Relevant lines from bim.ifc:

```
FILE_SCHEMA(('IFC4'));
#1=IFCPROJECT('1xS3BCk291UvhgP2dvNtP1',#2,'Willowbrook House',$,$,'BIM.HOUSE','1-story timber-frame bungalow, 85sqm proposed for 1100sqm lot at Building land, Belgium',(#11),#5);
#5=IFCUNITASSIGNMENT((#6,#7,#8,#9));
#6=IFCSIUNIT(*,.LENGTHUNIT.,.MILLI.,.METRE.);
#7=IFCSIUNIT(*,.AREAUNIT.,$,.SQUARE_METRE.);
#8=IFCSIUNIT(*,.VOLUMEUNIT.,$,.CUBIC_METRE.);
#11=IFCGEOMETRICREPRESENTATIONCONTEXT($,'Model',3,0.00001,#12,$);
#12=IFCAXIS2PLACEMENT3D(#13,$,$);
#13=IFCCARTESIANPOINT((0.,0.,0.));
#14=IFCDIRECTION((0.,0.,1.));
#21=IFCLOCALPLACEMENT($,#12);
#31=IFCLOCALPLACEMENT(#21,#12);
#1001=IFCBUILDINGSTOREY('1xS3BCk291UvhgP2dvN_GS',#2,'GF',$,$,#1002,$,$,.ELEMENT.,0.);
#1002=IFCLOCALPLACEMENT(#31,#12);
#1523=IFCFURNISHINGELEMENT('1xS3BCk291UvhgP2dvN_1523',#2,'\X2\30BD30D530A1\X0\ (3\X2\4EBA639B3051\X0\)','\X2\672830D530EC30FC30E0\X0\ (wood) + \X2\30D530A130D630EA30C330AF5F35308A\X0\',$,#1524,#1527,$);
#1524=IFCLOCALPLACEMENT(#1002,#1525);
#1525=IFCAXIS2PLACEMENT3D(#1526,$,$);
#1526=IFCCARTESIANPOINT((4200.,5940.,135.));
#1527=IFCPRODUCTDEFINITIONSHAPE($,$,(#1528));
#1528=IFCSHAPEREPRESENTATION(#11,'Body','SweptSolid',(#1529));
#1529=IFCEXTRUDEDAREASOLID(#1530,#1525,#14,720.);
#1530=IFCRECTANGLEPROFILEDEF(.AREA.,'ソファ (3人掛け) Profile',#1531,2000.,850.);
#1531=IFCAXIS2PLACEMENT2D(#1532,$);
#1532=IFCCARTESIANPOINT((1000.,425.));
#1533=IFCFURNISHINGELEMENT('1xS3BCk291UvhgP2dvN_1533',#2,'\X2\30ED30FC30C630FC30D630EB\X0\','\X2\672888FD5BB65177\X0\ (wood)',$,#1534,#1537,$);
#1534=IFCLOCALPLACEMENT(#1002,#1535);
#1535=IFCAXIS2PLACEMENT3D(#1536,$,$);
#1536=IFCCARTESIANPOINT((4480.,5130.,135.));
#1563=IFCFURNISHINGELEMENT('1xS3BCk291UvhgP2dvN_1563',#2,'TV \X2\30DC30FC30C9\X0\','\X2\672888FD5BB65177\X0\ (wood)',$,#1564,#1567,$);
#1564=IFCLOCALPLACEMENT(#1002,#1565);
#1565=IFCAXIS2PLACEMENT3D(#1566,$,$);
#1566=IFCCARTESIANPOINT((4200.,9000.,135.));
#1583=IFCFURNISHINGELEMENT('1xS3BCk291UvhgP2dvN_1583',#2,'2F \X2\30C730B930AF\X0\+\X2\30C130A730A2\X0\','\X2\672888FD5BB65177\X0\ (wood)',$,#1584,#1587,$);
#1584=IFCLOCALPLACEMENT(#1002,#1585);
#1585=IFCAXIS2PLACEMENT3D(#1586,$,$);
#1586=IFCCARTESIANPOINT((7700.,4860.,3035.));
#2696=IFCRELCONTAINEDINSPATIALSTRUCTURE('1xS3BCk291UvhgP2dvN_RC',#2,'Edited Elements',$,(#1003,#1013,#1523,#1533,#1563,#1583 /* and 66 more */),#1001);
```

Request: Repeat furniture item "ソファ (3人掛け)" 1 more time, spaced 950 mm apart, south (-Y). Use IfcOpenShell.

```python
import numpy as np
import ifcopenshell
import ifcopenshell.api.geometry
import ifcopenshell.api.root
import ifcopenshell.util.element
import ifcopenshell.util.placement
import ifcopenshell.util.unit

model = ifcopenshell.open("bim.ifc")
unit_scale = ifcopenshell.util.unit.calculate_unit_scale(model)


def reuse_history(source, copy):
    """copy_class also copies each property set's owner history, people and application; keep the originals."""
    for rel in copy.IsDefinedBy:
        if rel.is_a("IfcRelDefinesByProperties") and (history := rel.RelatingPropertyDefinition.OwnerHistory):
            rel.RelatingPropertyDefinition.OwnerHistory = source.OwnerHistory
            ifcopenshell.util.element.remove_deep2(model, history)


source = model.by_id(1523)
base = ifcopenshell.util.placement.get_local_placement(source.ObjectPlacement)
step = np.array([0.0, -1.0, 0.0]) * 0.95 / unit_scale

for i in range(1, 2):
    copy = ifcopenshell.api.root.copy_class(model, product=source)
    copy.Representation = ifcopenshell.util.element.copy_deep(
        model, source.Representation, exclude=["IfcGeometricRepresentationContext", "IfcRepresentationMap"]
    )
    reuse_history(source, copy)
    matrix = base.copy()
    matrix[:3, 3] += i * step
    print("added at", matrix[:3, 3].round(3) + 0.0)
    ifcopenshell.api.geometry.edit_object_placement(model, product=copy, matrix=matrix, is_si=False)

model.write("bim-out.ifc")
```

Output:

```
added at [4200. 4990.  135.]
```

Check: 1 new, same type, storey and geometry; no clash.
